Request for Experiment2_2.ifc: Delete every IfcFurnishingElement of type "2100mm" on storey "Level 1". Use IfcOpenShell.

First a look at what the model holds.

```python
import ifcopenshell
import ifcopenshell.util.element

model = ifcopenshell.open("Experiment2_2.ifc")
print(model.schema)
storey = next(s for s in model.by_type("IfcBuildingStorey") if s.Name == "Level 1")
furniture = [e for e in ifcopenshell.util.element.get_decomposition(storey) if e.is_a("IfcFurnishingElement")]
seen = {}
for e in furniture:
    element_type = ifcopenshell.util.element.get_type(e)
    name = element_type.Name if element_type not in (None, e) else None
    seen[name] = seen.get(name, 0) + 1
for name, count in sorted(seen.items(), key=str):
    print(count, "x", name)
```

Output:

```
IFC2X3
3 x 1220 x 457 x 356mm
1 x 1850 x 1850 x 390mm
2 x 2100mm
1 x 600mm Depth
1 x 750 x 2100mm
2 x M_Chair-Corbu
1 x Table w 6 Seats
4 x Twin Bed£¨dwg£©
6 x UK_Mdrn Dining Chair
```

```python
import ifcopenshell
import ifcopenshell.api.root
import ifcopenshell.util.element

model = ifcopenshell.open("Experiment2_2.ifc")

storey = next(s for s in model.by_type("IfcBuildingStorey") if s.Name == "Level 1")
furniture = [e for e in ifcopenshell.util.element.get_decomposition(storey) if e.is_a("IfcFurnishingElement")]
targets = [e for e in furniture if (t := ifcopenshell.util.element.get_type(e)) not in (None, e) and t.Name == "2100mm"]

for e in targets:
    ifcopenshell.api.root.remove_product(model, product=e)
print(len(targets), "removed")

model.write("Experiment2_2_rev.ifc")
```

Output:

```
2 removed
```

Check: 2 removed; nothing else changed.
